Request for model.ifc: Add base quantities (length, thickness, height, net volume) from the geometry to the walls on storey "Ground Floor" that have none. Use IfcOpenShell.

First a look at what the model holds.

```python
import ifcopenshell
import ifcopenshell.util.element
import ifcopenshell.util.unit

model = ifcopenshell.open("model.ifc")
print(model.schema)
for unit_type in ("LENGTHUNIT", "AREAUNIT", "VOLUMEUNIT"):
    print(unit_type, ifcopenshell.util.unit.calculate_unit_scale(model, unit_type))
storey = next(s for s in model.by_type("IfcBuildingStorey") if s.Name == "Ground Floor")
walls = [e for e in ifcopenshell.util.element.get_decomposition(storey) if e.is_a("IfcWall")]
for e in sorted(walls, key=lambda e: e.id()):
    print(e.id(), e.is_a(), e.Name, list(ifcopenshell.util.element.get_psets(e, qtos_only=True)), sep=" | ")
```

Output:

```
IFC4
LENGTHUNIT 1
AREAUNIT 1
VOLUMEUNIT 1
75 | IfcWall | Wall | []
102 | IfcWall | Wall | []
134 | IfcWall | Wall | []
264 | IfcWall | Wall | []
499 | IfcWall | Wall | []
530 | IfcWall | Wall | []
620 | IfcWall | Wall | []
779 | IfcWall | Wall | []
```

```python
import ifcopenshell
import ifcopenshell.api.pset
import ifcopenshell.geom
import ifcopenshell.util.element
import ifcopenshell.util.shape
import ifcopenshell.util.unit

model = ifcopenshell.open("model.ifc")
unit_scale = ifcopenshell.util.unit.calculate_unit_scale(model)
volume_scale = ifcopenshell.util.unit.calculate_unit_scale(model, "VOLUMEUNIT")
settings = ifcopenshell.geom.settings()

storey = next(s for s in model.by_type("IfcBuildingStorey") if s.Name == "Ground Floor")
walls = [e for e in ifcopenshell.util.element.get_decomposition(storey) if e.is_a("IfcWall")]

for e in sorted(walls, key=lambda e: e.id()):
    if ifcopenshell.util.element.get_psets(e, qtos_only=True, should_inherit=False):
        continue
    # Geometry comes back in metres, in the element's own axes.
    shape = ifcopenshell.geom.create_shape(settings, e)
    values = {
        "Length": ifcopenshell.util.shape.get_x(shape.geometry) / unit_scale,
        "Width": ifcopenshell.util.shape.get_y(shape.geometry) / unit_scale,
        "Height": ifcopenshell.util.shape.get_z(shape.geometry) / unit_scale,
        "NetVolume": ifcopenshell.util.shape.get_volume(shape.geometry) / volume_scale,
    }
    qto = ifcopenshell.api.pset.add_qto(model, product=e, name="Qto_WallBaseQuantities")
    ifcopenshell.api.pset.edit_qto(model, qto=qto, properties=values)
    print(e.id(), {k: round(v, 3) for k, v in values.items()})

model.write("model_rev.ifc")
```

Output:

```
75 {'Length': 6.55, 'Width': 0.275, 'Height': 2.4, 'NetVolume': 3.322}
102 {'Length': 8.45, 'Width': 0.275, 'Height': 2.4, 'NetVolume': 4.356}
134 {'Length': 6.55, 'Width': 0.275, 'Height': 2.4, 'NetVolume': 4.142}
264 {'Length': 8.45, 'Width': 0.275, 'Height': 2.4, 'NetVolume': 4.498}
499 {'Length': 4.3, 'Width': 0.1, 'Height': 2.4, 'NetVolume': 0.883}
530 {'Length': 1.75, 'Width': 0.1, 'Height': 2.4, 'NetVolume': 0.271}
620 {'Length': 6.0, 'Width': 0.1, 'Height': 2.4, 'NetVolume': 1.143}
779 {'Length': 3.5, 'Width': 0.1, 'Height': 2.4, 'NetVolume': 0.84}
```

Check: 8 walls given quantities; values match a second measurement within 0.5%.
